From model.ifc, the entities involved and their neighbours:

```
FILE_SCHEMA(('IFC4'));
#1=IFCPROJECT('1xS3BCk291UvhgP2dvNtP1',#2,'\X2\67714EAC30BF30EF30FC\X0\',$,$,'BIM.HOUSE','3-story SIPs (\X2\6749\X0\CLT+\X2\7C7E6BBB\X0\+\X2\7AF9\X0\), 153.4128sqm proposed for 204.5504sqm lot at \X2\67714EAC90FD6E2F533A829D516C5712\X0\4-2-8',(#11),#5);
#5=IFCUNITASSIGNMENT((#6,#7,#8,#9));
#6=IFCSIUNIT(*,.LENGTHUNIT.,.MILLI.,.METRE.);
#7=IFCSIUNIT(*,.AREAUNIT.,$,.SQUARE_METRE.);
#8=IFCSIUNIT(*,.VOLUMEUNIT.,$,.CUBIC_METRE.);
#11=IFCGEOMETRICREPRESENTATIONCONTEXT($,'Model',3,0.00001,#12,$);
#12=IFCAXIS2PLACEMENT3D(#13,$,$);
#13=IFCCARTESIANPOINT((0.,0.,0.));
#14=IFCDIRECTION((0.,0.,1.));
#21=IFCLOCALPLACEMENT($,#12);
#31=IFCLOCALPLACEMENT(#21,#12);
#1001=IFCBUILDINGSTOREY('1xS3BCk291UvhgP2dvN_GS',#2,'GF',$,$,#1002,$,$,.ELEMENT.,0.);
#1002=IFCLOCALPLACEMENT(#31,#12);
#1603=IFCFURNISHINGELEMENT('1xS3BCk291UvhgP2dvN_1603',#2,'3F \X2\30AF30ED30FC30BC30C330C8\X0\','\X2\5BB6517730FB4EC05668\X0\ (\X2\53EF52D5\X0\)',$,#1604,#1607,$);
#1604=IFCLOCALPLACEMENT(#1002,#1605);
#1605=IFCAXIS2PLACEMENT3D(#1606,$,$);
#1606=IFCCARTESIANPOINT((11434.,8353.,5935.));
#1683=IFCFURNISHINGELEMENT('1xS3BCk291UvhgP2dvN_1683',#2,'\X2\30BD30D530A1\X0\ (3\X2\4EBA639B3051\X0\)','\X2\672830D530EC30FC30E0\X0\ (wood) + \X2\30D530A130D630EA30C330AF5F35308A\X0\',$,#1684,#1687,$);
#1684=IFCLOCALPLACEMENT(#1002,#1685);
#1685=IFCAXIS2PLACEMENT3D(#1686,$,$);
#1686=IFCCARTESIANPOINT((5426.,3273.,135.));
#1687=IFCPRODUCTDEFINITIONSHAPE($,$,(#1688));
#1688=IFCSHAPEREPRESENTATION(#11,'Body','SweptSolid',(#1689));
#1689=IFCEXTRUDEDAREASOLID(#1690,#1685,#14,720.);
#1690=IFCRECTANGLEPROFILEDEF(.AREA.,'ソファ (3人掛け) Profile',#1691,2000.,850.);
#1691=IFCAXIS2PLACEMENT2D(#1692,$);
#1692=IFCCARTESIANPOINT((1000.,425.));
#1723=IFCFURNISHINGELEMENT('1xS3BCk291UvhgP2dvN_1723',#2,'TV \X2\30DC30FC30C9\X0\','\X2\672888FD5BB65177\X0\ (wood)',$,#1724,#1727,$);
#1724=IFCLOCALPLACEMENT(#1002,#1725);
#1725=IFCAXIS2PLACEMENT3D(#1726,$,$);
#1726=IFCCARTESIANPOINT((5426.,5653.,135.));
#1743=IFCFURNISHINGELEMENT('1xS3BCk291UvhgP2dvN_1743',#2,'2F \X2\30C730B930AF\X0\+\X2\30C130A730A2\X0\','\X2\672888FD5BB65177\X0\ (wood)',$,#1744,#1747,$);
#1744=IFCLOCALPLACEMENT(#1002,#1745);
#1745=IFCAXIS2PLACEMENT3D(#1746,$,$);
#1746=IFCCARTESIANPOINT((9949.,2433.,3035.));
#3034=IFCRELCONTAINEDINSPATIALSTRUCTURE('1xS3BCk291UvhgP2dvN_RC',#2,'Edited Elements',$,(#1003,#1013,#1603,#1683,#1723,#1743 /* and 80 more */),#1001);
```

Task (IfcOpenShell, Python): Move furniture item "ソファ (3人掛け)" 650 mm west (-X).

```python
import ifcopenshell
import ifcopenshell.api.geometry
import ifcopenshell.util.placement
import ifcopenshell.util.unit

model = ifcopenshell.open("model.ifc")
unit_scale = ifcopenshell.util.unit.calculate_unit_scale(model)

item = model.by_guid("1xS3BCk291UvhgP2dvN_1683")
matrix = ifcopenshell.util.placement.get_local_placement(item.ObjectPlacement)
matrix[0, 3] -= 0.65 / unit_scale
ifcopenshell.api.geometry.edit_object_placement(model, product=item, matrix=matrix, is_si=False)

print(ifcopenshell.util.placement.get_local_placement(item.ObjectPlacement).round(3) + 0.0)

model.write("model_updated.ifc")
```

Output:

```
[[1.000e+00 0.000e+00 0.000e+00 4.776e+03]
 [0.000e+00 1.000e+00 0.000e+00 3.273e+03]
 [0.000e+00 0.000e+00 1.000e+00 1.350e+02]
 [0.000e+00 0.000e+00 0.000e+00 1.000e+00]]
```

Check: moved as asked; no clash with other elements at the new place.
